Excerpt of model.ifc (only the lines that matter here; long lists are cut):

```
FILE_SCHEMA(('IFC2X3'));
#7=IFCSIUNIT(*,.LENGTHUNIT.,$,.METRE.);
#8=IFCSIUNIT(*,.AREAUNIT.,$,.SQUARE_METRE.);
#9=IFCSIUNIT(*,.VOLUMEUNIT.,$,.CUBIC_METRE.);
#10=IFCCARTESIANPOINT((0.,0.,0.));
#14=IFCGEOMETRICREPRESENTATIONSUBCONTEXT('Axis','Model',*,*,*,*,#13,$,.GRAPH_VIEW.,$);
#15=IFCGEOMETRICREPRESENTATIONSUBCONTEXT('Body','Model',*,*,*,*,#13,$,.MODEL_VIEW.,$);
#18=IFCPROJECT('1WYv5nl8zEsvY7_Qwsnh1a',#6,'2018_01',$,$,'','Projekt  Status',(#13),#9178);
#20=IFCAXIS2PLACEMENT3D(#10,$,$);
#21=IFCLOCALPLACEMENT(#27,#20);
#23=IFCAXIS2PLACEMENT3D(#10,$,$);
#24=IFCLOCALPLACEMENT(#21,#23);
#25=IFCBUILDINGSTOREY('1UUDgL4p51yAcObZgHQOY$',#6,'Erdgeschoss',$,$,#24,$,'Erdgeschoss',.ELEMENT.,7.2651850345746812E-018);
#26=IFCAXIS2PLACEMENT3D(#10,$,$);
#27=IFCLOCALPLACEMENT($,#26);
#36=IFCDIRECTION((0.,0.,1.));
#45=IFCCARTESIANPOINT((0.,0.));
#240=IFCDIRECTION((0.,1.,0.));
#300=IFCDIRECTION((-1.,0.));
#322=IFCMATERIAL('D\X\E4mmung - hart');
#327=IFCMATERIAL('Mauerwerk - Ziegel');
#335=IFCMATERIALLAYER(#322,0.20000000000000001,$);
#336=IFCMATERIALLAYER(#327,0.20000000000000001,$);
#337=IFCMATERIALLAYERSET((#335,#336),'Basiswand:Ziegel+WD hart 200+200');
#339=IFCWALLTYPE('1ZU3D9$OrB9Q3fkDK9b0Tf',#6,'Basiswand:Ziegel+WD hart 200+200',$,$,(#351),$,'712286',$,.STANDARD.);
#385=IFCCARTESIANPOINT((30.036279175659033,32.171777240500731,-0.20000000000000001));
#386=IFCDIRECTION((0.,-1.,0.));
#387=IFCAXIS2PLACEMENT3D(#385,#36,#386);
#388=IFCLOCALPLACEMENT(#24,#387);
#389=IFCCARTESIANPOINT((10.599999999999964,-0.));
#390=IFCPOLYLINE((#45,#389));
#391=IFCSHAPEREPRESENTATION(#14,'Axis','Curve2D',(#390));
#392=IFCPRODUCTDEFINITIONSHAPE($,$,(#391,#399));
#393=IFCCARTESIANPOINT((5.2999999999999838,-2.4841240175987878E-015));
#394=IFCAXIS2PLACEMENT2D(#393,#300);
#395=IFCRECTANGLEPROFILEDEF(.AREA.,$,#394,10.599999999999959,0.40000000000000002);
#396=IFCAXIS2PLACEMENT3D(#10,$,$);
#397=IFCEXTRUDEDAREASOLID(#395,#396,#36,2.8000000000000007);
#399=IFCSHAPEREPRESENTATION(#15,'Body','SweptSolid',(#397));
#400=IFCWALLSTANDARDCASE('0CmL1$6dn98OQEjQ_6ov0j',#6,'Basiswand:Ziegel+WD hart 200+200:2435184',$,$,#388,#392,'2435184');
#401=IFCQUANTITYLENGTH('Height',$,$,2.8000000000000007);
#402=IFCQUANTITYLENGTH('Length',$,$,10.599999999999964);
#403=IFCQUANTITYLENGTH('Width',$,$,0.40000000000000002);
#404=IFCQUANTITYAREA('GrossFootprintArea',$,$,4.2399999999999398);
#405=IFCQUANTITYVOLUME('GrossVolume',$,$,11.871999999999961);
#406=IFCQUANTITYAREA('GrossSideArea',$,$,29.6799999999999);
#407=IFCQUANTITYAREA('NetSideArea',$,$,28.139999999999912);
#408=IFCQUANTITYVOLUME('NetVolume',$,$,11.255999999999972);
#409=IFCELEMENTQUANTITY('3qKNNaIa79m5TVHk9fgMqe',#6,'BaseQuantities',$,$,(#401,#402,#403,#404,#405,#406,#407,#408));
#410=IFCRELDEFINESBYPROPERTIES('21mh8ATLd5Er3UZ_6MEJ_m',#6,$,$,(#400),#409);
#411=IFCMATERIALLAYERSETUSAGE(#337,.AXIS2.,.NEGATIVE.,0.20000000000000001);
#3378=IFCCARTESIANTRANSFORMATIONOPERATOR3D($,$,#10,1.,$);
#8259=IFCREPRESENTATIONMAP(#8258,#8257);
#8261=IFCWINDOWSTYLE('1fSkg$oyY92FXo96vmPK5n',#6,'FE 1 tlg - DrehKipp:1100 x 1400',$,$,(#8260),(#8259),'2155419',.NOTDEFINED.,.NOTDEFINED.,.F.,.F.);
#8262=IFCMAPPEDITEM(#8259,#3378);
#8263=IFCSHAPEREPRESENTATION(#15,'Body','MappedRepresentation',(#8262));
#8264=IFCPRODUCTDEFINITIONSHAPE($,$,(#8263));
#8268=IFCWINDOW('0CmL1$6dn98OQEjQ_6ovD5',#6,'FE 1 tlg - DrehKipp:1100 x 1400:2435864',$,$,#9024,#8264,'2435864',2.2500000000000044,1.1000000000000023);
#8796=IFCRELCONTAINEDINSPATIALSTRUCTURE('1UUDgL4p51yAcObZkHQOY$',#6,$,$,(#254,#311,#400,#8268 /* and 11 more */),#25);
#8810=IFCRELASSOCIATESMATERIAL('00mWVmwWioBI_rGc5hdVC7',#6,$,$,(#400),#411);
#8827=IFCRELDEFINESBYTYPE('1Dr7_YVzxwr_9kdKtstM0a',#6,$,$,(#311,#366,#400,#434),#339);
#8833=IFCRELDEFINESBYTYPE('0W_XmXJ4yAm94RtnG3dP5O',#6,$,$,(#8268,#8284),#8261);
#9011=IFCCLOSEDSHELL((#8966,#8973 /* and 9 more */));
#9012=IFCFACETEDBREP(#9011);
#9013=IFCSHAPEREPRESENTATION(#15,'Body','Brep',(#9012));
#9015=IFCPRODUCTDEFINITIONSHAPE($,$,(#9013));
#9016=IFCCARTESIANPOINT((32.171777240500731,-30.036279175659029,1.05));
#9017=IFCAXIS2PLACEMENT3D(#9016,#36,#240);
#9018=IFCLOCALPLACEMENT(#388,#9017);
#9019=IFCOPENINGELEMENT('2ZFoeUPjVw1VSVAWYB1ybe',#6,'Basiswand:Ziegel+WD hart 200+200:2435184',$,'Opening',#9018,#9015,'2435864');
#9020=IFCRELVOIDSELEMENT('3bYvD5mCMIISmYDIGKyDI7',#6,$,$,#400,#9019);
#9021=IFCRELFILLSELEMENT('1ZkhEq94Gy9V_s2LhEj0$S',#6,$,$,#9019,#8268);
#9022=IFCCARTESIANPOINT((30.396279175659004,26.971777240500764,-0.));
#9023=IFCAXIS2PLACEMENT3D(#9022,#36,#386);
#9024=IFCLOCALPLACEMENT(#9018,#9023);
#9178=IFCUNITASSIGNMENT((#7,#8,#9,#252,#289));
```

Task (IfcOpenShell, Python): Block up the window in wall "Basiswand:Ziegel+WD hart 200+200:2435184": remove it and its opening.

```python
import ifcopenshell
import ifcopenshell.api.feature
import ifcopenshell.api.pset
import ifcopenshell.api.root
import ifcopenshell.geom
import ifcopenshell.util.element
import ifcopenshell.util.shape
import ifcopenshell.util.unit

model = ifcopenshell.open("model.ifc")
area_scale = ifcopenshell.util.unit.calculate_unit_scale(model, "AREAUNIT")
volume_scale = ifcopenshell.util.unit.calculate_unit_scale(model, "VOLUMEUNIT")
settings = ifcopenshell.geom.settings()


def volume(element):
    """Net volume in cubic metres, openings subtracted."""
    shape = ifcopenshell.geom.create_shape(settings, element)
    return ifcopenshell.util.shape.get_volume(shape.geometry)


window = model.by_id(8268)
opening = window.FillsVoids[0].RelatingOpeningElement
wall = opening.VoidsElements[0].RelatingBuildingElement
before = volume(wall)

ifcopenshell.api.root.remove_product(model, product=window)
ifcopenshell.api.feature.remove_feature(model, feature=opening)

after = volume(wall)
thickness = 0.4  # wall thickness in metres

# Update the wall's stored quantities.
qto = model.by_id(ifcopenshell.util.element.get_pset(wall, "BaseQuantities", should_inherit=False)["id"])
ifcopenshell.api.pset.edit_qto(model, qto=qto, properties={
    "NetSideArea": after / thickness / area_scale,
    "NetVolume": after / volume_scale,
})

print(f"wall volume {before:.3f} -> {after:.3f} m3")

model.write("model-out.ifc")
```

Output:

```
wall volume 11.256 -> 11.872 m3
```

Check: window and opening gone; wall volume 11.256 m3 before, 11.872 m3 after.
